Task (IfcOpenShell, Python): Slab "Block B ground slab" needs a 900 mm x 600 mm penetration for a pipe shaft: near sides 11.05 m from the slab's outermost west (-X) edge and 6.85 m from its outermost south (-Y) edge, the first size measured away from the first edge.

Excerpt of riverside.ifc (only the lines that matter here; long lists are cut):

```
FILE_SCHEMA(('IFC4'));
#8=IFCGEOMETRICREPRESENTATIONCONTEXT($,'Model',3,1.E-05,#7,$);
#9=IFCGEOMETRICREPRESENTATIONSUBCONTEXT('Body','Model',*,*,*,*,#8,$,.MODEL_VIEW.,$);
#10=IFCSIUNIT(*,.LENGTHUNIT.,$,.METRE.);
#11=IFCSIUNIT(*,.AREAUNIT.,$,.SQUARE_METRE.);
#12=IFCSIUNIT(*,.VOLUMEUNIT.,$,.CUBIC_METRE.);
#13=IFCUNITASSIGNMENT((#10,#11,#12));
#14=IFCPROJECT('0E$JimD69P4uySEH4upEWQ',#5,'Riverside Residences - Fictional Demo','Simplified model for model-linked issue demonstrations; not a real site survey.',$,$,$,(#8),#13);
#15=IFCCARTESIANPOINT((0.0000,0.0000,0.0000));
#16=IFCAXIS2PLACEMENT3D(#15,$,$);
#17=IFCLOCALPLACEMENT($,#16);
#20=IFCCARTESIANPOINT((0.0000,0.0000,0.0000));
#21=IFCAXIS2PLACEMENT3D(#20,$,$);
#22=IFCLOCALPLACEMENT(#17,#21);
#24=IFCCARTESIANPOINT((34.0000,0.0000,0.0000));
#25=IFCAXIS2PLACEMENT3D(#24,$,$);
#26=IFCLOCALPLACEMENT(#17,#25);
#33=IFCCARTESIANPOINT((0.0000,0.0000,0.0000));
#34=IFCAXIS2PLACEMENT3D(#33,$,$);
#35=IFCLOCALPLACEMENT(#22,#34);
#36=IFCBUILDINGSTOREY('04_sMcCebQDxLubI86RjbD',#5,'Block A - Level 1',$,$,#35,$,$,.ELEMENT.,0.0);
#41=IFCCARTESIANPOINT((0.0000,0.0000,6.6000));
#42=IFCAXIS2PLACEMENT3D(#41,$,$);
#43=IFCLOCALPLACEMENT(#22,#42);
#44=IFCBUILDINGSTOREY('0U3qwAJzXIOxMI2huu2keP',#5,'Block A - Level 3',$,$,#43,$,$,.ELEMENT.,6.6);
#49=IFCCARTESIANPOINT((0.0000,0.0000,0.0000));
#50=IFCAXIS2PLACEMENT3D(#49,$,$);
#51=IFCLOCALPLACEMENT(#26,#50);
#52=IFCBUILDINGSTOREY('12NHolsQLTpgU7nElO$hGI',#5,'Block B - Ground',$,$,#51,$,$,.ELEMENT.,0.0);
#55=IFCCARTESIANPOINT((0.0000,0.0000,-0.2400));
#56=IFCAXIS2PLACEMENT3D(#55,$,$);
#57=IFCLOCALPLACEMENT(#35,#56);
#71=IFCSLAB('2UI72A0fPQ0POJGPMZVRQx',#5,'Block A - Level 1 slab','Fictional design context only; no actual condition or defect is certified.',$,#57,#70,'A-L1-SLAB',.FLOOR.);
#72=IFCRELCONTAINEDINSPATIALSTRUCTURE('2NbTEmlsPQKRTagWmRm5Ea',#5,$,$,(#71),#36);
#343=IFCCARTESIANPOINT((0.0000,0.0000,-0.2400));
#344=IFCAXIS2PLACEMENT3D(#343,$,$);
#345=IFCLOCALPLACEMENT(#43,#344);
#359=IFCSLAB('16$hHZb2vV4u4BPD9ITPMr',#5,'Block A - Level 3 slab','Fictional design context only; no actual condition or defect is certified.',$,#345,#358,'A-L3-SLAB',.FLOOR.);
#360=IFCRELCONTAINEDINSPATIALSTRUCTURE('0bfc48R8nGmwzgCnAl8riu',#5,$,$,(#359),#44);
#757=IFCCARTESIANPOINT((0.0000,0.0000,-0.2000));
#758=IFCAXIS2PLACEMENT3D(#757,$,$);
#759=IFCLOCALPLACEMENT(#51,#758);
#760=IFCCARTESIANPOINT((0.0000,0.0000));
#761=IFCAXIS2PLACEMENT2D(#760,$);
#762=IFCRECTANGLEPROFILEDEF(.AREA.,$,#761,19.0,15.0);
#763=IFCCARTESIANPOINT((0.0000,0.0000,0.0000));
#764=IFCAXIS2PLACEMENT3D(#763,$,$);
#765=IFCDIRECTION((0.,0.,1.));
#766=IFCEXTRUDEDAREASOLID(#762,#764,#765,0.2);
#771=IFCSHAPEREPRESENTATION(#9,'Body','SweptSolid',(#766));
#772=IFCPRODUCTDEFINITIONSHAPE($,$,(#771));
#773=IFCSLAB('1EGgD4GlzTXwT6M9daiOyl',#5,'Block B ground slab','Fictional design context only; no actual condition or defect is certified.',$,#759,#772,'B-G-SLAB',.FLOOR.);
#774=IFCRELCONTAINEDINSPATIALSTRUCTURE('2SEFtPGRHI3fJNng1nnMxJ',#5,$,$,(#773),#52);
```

```python
import numpy as np
import ifcopenshell
import ifcopenshell.api.feature
import ifcopenshell.api.geometry
import ifcopenshell.api.root
import ifcopenshell.geom
import ifcopenshell.util.placement
import ifcopenshell.util.representation
import ifcopenshell.util.shape
import ifcopenshell.util.unit

model = ifcopenshell.open("riverside.ifc")
unit_scale = ifcopenshell.util.unit.calculate_unit_scale(model)
settings = ifcopenshell.geom.settings()


def volume(element):
    """Net volume in cubic metres, openings subtracted."""
    shape = ifcopenshell.geom.create_shape(settings, element)
    return ifcopenshell.util.shape.get_volume(shape.geometry)


slab = model.by_id(773)
before = volume(slab)

# Extent in the slab's own axes, in metres. The edges named are its -X and -Y sides.
slab_shape = ifcopenshell.geom.create_shape(settings, slab)
vertices = ifcopenshell.util.shape.get_vertices(slab_shape.geometry)
x_min, y_min, bottom = vertices.min(axis=0)
top = vertices[:, 2].max()

opening = ifcopenshell.api.root.create_entity(model, ifc_class="IfcOpeningElement", name="Pipe shaft opening", predefined_type="OPENING")
context = ifcopenshell.util.representation.get_context(model, "Model", "Body", "MODEL_VIEW")
width, depth = 0.9, 0.6
outline = [(0.0, 0.0), (width, 0.0), (width, depth), (0.0, depth), (0.0, 0.0)]
# Overshoot both faces by 50 mm so the cut is clean.
shape = ifcopenshell.api.geometry.add_slab_representation(
    model, context=context, depth=top - bottom + 0.1, polyline=outline
)
ifcopenshell.api.geometry.assign_representation(model, product=opening, representation=shape)

matrix = ifcopenshell.util.placement.get_local_placement(slab.ObjectPlacement)
matrix[:, 3] = matrix @ np.append(np.array([x_min + 11.05, y_min + 6.85, bottom - 0.05]) / unit_scale, 1.0)
ifcopenshell.api.geometry.edit_object_placement(model, product=opening, matrix=matrix, is_si=False)
ifcopenshell.api.feature.add_feature(model, feature=opening, element=slab)

after = volume(slab)

print(f"slab volume {before:.3f} -> {after:.3f} m3")

model.write("riverside_updated.ifc")
```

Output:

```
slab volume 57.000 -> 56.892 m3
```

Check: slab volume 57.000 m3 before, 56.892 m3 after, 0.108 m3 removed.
